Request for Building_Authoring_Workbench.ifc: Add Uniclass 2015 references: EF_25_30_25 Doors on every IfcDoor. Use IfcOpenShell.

First a look at what the model holds.

```python
import ifcopenshell

model = ifcopenshell.open("Building_Authoring_Workbench.ifc")
print(model.schema)
print("classifications:", [c.Name for c in model.by_type("IfcClassification")])
for ifc_class in ("IfcDoor", "IfcRoof", "IfcStair", "IfcWall", "IfcWindow"):
    print(ifc_class, len(model.by_type(ifc_class)))
```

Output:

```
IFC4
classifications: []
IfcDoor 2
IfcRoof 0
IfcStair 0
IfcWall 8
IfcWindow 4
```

```python
import ifcopenshell
import ifcopenshell.api.classification

model = ifcopenshell.open("Building_Authoring_Workbench.ifc")

system = ifcopenshell.api.classification.add_classification(model, classification="Uniclass 2015")

codes = {
    "IfcDoor": ("EF_25_30_25", "Doors"),
}
for ifc_class, (code, name) in codes.items():
    products = model.by_type(ifc_class)
    ifcopenshell.api.classification.add_reference(
        model, products=products, classification=system, identification=code, name=name
    )
    print(code, len(products))

model.write("Building_Authoring_Workbench_rev.ifc")
```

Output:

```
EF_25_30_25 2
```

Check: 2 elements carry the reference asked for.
